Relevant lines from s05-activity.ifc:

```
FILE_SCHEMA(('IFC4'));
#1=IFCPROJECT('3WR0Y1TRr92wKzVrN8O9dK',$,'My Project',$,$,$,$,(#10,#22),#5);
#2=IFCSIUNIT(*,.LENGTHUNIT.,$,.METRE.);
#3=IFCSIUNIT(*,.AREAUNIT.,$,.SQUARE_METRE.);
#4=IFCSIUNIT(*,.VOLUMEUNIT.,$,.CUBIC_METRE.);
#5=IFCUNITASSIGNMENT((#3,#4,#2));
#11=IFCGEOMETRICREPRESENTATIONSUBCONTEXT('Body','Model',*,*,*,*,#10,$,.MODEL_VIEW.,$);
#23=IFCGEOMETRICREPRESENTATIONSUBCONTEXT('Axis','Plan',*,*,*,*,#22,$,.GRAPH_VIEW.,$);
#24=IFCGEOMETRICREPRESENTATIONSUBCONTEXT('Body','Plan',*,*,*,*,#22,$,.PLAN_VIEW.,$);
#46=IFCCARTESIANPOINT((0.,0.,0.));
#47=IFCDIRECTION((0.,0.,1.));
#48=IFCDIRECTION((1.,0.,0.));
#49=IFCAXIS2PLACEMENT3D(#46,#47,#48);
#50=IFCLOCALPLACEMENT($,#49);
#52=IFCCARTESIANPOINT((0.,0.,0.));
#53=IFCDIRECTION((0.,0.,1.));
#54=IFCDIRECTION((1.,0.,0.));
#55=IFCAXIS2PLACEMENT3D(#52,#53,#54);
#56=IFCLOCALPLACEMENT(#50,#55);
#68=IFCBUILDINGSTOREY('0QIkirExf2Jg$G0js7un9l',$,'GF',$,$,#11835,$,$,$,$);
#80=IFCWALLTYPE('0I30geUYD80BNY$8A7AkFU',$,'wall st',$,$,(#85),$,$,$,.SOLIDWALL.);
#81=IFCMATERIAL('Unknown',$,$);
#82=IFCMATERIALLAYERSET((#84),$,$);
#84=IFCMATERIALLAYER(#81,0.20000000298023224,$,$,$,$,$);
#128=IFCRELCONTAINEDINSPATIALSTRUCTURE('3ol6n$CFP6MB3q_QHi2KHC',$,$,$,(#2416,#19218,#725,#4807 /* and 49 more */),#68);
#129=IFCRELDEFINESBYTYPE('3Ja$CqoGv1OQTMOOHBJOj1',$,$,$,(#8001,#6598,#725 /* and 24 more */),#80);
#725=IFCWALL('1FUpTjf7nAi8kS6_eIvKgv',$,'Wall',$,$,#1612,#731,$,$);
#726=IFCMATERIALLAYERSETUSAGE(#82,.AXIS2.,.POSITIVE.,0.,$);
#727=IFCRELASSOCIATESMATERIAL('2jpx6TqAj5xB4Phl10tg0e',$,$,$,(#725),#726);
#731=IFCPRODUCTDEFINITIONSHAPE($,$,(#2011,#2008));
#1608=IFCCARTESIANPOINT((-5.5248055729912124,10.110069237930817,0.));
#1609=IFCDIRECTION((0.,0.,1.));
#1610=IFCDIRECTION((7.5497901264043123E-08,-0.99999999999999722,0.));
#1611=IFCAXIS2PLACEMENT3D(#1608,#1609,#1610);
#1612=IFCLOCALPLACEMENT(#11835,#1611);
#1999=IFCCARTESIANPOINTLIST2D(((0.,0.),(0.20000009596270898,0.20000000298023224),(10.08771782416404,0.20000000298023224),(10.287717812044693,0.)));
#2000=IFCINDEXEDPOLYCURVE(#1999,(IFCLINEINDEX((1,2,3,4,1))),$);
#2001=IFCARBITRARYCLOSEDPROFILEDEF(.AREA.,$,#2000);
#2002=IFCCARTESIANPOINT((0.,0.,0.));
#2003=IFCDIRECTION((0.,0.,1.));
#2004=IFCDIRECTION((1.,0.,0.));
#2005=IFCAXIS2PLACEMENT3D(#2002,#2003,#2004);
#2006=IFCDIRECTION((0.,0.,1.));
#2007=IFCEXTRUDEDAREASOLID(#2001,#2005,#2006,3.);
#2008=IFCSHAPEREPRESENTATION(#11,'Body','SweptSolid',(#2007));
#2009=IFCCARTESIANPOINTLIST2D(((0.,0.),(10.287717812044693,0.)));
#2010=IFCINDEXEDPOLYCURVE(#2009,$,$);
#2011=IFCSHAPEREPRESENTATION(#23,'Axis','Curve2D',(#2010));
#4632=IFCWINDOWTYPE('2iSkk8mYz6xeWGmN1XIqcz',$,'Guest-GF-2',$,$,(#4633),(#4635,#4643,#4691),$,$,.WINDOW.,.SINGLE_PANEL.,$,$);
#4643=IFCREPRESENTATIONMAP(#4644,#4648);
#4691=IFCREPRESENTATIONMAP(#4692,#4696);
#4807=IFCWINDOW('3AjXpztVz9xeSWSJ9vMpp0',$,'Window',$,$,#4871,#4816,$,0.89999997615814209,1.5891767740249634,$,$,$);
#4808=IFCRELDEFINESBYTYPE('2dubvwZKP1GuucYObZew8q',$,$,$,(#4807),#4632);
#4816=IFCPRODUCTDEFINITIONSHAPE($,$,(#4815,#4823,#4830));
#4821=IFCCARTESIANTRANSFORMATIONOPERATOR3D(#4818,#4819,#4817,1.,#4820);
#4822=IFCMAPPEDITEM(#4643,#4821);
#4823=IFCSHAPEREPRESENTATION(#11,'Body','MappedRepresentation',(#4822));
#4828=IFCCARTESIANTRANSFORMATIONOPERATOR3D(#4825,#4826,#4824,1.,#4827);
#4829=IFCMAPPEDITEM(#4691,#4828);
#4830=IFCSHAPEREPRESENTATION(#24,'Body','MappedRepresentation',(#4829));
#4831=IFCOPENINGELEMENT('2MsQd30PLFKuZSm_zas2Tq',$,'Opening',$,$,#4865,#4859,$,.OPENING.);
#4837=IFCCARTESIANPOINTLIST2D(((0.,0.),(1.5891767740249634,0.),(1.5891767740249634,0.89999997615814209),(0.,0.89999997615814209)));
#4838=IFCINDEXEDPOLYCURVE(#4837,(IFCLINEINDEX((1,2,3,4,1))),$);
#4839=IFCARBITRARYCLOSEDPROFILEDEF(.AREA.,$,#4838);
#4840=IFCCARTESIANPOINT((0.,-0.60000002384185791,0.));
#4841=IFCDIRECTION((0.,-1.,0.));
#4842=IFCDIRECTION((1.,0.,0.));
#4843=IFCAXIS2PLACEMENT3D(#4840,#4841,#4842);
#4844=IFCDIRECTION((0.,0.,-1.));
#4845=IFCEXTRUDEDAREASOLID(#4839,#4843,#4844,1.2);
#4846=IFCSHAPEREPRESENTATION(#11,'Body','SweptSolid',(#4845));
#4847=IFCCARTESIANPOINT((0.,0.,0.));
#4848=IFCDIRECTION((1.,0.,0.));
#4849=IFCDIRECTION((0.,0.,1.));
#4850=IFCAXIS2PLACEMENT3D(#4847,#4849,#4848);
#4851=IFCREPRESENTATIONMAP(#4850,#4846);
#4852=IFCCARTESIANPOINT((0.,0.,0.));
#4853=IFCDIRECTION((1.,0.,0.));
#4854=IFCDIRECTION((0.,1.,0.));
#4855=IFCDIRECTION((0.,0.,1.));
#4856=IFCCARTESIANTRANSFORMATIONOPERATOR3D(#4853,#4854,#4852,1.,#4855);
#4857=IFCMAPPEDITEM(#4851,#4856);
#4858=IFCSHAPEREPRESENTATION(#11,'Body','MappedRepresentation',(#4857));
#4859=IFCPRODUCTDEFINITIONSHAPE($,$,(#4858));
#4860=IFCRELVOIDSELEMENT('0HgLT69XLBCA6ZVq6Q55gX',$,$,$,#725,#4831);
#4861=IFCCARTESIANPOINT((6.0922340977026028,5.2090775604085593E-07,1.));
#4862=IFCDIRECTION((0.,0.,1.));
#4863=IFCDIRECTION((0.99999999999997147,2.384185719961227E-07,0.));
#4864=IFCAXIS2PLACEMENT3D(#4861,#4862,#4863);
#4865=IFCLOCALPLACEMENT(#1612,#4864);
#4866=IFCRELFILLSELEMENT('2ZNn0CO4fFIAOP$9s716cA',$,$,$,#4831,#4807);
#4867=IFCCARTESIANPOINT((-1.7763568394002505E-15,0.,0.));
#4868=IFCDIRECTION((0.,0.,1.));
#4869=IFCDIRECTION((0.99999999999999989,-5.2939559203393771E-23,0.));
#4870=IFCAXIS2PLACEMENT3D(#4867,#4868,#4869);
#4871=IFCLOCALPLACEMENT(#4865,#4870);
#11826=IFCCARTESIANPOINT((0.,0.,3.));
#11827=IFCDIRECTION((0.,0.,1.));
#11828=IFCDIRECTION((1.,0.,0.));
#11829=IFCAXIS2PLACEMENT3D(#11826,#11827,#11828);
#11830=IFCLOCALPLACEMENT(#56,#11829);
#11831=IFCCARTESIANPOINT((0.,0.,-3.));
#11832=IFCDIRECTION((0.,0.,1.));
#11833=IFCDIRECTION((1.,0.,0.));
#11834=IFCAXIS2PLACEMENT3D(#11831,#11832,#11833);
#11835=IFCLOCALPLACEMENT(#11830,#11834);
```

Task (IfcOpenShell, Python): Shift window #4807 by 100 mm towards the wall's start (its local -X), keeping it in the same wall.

```python
import ifcopenshell
import ifcopenshell.api.geometry
import ifcopenshell.util.placement

model = ifcopenshell.open("s05-activity.ifc")

window = model.by_guid("3AjXpztVz9xeSWSJ9vMpp0")
opening = window.FillsVoids[0].RelatingOpeningElement
wall = opening.VoidsElements[0].RelatingBuildingElement

wall_matrix = ifcopenshell.util.placement.get_local_placement(wall.ObjectPlacement)
shift = wall_matrix[:3, 0] * -0.1
before = ifcopenshell.util.placement.get_local_placement(window.ObjectPlacement)[:3, 3].copy()

# The window is placed relative to its opening, so it follows when the opening moves.
matrix = ifcopenshell.util.placement.get_local_placement(opening.ObjectPlacement)
matrix[:3, 3] += shift
ifcopenshell.api.geometry.edit_object_placement(
    model, product=opening, matrix=matrix, is_si=False, should_transform_children=True
)

after = ifcopenshell.util.placement.get_local_placement(window.ObjectPlacement)[:3, 3]
print("window moved by", (after - before).round(3) + 0.0)

model.write("s05-activity_v2.ifc")
```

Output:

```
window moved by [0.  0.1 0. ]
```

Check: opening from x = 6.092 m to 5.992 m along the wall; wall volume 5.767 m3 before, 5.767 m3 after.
